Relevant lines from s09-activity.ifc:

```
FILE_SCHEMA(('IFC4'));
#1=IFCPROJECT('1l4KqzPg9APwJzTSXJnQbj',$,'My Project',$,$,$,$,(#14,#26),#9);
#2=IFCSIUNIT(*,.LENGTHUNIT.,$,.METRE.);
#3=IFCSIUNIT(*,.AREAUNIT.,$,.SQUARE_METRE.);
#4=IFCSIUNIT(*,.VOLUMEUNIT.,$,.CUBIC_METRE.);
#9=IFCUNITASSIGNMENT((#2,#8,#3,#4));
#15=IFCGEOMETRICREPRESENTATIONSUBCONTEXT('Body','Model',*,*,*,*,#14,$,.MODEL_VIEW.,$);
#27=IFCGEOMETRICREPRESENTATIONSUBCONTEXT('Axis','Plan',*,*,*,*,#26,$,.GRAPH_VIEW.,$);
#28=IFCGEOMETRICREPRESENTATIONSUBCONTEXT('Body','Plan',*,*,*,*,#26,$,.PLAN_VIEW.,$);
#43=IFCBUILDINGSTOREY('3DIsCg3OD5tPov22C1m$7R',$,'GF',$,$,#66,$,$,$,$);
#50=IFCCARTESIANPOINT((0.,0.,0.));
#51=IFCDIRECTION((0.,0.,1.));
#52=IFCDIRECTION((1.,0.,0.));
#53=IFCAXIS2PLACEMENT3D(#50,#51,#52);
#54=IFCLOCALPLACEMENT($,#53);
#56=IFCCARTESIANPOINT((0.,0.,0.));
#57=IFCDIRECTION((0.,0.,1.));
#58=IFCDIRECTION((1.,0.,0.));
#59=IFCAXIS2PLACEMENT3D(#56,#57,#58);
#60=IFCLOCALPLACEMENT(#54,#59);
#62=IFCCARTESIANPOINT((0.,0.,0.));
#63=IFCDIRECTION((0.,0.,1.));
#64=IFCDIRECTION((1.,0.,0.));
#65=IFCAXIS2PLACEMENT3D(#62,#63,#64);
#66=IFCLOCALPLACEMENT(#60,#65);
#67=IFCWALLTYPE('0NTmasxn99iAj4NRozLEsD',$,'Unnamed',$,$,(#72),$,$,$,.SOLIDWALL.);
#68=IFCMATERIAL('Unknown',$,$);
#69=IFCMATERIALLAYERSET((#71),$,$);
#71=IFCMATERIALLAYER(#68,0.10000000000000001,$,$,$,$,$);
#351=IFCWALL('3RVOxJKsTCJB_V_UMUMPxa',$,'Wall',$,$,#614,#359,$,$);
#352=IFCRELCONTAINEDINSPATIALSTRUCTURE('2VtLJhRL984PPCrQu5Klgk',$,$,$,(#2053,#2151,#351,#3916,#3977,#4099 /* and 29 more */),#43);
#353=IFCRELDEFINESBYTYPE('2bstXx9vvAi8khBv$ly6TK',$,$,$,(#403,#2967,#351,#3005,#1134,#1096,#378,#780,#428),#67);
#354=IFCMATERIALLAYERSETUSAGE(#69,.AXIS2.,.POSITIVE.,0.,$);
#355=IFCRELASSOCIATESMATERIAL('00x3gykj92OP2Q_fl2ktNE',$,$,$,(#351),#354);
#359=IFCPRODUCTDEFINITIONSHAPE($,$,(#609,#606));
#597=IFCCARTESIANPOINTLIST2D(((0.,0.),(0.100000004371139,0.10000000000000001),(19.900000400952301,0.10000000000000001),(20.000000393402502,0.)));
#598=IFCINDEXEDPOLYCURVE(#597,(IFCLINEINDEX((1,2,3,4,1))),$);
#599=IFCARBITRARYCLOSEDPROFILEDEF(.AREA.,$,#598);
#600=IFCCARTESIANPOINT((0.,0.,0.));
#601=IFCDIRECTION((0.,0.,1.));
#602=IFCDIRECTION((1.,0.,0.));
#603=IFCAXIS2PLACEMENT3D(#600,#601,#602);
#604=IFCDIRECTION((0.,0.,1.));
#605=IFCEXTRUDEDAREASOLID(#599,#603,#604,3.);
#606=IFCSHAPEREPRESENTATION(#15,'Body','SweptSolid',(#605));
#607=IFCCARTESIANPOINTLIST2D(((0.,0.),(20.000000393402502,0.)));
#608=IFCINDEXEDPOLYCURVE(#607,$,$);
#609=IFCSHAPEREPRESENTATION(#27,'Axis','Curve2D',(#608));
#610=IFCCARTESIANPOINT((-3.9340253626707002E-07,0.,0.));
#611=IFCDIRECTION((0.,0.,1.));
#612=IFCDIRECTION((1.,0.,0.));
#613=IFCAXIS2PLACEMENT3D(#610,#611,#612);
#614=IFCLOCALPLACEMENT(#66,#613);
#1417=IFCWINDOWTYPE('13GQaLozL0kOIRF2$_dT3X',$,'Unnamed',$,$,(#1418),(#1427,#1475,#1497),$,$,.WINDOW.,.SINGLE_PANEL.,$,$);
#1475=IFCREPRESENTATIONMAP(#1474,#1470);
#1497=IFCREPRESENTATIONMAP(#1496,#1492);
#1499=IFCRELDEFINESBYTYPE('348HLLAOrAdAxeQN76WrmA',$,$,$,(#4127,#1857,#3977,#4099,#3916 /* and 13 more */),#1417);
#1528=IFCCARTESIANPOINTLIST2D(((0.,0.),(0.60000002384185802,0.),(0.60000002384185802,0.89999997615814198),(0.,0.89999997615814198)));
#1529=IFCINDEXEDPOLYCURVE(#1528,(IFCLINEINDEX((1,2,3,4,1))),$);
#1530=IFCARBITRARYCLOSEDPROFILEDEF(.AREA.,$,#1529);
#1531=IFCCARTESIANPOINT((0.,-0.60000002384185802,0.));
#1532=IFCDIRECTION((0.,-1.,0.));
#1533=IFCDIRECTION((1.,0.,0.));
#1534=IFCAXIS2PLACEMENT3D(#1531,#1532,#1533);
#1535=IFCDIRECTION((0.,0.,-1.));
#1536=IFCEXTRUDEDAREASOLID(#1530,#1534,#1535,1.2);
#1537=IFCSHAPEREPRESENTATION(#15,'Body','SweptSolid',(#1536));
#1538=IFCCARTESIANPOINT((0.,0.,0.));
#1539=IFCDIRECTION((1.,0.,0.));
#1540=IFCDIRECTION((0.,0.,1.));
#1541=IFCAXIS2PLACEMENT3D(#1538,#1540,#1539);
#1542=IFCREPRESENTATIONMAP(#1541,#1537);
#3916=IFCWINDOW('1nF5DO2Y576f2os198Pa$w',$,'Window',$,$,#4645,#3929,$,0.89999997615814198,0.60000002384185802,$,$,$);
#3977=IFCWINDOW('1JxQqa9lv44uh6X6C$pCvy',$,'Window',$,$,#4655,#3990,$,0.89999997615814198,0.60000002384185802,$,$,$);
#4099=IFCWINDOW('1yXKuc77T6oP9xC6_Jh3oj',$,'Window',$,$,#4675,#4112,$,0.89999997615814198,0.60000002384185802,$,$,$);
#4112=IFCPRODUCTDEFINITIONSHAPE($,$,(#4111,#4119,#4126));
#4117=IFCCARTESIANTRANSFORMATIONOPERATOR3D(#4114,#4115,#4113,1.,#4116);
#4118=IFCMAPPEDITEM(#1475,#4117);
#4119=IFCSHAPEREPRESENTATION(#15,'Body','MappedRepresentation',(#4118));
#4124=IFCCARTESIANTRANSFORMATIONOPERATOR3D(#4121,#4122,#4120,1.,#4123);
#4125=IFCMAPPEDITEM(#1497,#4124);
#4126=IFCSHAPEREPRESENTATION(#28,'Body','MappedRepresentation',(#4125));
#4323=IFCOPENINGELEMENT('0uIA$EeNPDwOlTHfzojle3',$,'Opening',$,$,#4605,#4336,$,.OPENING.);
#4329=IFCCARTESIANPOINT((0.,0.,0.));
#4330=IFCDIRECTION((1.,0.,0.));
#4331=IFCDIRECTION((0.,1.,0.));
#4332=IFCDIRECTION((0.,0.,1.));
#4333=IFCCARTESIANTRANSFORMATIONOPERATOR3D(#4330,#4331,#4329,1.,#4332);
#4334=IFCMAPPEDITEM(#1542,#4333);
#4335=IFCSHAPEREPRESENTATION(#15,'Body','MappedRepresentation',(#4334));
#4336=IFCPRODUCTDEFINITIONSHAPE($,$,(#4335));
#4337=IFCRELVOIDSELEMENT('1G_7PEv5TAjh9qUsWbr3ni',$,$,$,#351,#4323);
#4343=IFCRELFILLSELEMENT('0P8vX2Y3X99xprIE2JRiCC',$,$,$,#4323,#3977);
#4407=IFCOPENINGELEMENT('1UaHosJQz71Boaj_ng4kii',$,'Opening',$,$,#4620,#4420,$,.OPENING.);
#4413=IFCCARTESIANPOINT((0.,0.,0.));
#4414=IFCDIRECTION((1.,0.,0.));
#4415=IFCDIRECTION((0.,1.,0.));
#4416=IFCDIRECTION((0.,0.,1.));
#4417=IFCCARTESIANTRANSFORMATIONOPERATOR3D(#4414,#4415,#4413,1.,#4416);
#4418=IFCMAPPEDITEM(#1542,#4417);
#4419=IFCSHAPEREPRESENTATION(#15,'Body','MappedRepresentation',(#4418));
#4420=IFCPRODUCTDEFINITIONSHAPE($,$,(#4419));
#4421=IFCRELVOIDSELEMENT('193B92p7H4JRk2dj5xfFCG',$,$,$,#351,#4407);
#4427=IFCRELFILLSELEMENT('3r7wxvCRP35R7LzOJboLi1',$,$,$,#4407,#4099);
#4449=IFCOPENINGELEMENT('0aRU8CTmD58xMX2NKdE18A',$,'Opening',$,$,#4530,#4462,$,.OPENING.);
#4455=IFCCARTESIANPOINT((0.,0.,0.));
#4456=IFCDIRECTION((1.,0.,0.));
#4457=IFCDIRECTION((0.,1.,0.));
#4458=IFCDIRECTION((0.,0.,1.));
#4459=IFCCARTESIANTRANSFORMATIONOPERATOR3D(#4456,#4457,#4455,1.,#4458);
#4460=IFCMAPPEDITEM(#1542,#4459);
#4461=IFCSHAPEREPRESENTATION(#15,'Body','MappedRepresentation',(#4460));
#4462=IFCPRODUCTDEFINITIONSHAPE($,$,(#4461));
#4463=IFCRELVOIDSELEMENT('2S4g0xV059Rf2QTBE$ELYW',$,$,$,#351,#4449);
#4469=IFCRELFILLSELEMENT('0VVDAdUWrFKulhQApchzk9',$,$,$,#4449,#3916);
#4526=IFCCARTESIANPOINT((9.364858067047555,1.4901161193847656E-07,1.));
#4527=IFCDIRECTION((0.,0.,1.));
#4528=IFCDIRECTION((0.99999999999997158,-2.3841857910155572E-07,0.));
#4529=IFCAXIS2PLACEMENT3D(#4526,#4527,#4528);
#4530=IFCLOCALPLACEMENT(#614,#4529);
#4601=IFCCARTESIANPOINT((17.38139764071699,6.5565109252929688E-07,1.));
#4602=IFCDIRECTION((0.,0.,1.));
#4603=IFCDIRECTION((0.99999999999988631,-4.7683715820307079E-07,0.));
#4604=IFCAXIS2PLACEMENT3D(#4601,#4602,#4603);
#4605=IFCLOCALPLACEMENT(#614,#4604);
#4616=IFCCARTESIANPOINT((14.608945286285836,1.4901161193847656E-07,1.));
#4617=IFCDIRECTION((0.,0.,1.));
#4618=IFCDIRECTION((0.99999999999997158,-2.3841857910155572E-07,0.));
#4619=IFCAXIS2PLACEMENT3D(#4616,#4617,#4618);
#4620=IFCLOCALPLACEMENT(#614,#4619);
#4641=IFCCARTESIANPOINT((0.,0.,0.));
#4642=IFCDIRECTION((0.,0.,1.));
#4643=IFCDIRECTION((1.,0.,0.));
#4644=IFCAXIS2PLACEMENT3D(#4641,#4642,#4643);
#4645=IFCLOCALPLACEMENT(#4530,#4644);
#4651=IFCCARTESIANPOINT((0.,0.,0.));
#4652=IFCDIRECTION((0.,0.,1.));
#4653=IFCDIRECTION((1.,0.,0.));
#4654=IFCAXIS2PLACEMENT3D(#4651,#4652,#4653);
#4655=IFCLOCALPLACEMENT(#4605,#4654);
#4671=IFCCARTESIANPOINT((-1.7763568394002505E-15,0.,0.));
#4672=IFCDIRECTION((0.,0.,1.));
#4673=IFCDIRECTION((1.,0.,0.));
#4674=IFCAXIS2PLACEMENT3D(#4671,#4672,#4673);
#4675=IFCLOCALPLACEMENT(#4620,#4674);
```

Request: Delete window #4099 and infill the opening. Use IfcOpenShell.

```python
import ifcopenshell
import ifcopenshell.api.feature
import ifcopenshell.api.root
import ifcopenshell.geom
import ifcopenshell.util.shape

model = ifcopenshell.open("s09-activity.ifc")
settings = ifcopenshell.geom.settings()


def volume(element):
    """Net volume in cubic metres, openings subtracted."""
    shape = ifcopenshell.geom.create_shape(settings, element)
    return ifcopenshell.util.shape.get_volume(shape.geometry)


window = model.by_id(4099)
opening = window.FillsVoids[0].RelatingOpeningElement
wall = opening.VoidsElements[0].RelatingBuildingElement
before = volume(wall)

ifcopenshell.api.root.remove_product(model, product=window)
ifcopenshell.api.feature.remove_feature(model, feature=opening)

after = volume(wall)

print(f"wall volume {before:.3f} -> {after:.3f} m3")

model.write("s09-activity-out.ifc")
```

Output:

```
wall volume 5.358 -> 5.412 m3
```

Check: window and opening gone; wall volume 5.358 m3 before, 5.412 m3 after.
